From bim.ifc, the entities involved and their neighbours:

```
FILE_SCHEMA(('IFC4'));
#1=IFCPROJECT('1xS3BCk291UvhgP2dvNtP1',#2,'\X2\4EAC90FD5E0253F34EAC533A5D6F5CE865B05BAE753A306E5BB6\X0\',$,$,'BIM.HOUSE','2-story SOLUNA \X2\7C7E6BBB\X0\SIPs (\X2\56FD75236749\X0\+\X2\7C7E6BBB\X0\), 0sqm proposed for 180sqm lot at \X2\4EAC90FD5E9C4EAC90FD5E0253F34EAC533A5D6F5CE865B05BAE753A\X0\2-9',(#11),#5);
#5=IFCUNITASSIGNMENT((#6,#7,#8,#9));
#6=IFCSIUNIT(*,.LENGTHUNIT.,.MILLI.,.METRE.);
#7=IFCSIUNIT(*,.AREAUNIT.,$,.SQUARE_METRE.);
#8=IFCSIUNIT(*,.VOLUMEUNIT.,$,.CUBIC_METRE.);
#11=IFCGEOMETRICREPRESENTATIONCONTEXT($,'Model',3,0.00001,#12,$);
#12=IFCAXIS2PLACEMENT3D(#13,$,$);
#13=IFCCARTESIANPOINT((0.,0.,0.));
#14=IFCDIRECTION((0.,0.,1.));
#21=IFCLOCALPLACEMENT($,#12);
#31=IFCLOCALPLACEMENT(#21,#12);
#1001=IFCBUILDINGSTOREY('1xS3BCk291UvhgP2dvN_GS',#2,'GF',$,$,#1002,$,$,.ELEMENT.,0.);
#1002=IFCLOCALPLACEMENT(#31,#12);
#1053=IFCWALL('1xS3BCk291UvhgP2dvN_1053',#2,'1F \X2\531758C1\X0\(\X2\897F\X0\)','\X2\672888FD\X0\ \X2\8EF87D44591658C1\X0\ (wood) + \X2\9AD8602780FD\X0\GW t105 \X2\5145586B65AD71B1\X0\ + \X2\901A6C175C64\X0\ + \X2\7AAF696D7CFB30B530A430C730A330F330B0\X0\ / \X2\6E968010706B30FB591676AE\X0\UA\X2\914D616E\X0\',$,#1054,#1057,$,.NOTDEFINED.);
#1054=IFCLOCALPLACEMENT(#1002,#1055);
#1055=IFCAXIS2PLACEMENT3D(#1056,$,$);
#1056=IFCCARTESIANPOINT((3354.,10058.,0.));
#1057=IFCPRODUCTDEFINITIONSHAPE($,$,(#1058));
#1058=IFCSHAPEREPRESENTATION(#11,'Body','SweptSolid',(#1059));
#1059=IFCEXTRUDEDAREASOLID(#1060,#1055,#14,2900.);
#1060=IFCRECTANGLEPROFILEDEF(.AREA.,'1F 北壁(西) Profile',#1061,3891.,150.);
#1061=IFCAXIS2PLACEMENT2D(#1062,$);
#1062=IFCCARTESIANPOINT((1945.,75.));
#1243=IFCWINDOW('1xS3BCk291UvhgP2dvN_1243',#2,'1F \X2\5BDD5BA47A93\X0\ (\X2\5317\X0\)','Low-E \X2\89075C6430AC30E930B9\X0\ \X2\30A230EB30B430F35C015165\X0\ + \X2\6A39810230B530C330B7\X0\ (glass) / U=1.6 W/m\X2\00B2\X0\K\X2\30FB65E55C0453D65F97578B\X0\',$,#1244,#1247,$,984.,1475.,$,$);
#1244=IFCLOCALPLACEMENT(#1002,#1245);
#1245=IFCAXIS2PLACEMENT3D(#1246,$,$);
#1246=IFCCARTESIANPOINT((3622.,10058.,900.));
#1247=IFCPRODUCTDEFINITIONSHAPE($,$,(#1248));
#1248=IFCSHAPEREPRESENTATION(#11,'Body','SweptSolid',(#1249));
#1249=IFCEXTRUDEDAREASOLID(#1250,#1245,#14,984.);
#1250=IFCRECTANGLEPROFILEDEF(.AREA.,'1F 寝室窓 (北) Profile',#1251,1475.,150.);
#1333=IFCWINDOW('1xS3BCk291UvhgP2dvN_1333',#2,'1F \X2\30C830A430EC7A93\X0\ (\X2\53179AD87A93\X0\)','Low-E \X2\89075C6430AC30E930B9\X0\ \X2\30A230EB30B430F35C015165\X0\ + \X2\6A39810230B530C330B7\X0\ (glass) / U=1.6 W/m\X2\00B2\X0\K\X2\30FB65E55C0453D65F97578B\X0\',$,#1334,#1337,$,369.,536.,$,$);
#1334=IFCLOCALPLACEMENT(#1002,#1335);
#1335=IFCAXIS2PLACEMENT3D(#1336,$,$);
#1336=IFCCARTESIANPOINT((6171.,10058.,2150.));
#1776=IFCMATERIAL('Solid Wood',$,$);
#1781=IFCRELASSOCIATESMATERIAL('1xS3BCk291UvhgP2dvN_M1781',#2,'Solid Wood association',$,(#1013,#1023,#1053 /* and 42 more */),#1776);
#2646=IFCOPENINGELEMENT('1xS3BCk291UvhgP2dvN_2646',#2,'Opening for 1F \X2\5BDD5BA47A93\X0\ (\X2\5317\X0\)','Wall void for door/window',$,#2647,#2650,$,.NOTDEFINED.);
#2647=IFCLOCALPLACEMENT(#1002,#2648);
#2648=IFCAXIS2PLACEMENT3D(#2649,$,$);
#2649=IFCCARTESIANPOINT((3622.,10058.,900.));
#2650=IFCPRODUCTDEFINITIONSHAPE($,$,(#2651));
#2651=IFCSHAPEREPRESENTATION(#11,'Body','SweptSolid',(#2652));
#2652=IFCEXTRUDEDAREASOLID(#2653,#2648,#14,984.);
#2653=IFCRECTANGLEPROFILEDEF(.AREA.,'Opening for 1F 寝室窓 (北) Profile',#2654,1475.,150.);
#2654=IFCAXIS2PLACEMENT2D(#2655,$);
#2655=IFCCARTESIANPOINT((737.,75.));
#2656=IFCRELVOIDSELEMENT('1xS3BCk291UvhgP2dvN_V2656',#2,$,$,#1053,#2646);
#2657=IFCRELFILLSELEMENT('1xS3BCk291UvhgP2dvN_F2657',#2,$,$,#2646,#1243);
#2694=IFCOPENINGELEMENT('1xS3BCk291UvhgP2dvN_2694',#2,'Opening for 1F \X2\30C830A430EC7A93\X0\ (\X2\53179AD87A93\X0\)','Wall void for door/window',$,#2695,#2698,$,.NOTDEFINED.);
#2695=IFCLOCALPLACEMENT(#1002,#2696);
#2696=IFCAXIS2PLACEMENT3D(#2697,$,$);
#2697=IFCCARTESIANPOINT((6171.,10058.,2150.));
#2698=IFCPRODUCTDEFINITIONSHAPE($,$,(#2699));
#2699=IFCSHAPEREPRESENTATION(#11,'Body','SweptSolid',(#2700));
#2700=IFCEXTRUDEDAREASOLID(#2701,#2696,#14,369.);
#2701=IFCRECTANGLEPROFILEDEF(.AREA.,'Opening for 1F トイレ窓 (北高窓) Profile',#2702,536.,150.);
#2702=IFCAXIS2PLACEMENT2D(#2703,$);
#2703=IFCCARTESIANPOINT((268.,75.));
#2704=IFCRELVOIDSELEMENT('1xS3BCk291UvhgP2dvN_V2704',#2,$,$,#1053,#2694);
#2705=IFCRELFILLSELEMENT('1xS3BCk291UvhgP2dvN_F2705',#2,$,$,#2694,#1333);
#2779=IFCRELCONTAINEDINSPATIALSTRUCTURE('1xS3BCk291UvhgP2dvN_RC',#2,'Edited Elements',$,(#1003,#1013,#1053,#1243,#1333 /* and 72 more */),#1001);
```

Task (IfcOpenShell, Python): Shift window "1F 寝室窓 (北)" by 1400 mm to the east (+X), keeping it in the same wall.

```python
import ifcopenshell
import ifcopenshell.api.geometry
import ifcopenshell.util.placement

model = ifcopenshell.open("bim.ifc")

window = model.by_guid("1xS3BCk291UvhgP2dvN_1243")
opening = window.FillsVoids[0].RelatingOpeningElement
wall = opening.VoidsElements[0].RelatingBuildingElement

wall_matrix = ifcopenshell.util.placement.get_local_placement(wall.ObjectPlacement)
shift = wall_matrix[:3, 0] * 1400.0
before = ifcopenshell.util.placement.get_local_placement(window.ObjectPlacement)[:3, 3].copy()

# The window is not placed relative to its opening, so move both.
for product in (opening, window):
    matrix = ifcopenshell.util.placement.get_local_placement(product.ObjectPlacement)
    matrix[:3, 3] += shift
    ifcopenshell.api.geometry.edit_object_placement(model, product=product, matrix=matrix, is_si=False)

after = ifcopenshell.util.placement.get_local_placement(window.ObjectPlacement)[:3, 3]
print("window moved by", (after - before).round(3) + 0.0)

model.write("bim_rev.ifc")
```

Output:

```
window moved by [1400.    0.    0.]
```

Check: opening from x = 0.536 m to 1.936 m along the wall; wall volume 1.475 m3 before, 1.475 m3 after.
